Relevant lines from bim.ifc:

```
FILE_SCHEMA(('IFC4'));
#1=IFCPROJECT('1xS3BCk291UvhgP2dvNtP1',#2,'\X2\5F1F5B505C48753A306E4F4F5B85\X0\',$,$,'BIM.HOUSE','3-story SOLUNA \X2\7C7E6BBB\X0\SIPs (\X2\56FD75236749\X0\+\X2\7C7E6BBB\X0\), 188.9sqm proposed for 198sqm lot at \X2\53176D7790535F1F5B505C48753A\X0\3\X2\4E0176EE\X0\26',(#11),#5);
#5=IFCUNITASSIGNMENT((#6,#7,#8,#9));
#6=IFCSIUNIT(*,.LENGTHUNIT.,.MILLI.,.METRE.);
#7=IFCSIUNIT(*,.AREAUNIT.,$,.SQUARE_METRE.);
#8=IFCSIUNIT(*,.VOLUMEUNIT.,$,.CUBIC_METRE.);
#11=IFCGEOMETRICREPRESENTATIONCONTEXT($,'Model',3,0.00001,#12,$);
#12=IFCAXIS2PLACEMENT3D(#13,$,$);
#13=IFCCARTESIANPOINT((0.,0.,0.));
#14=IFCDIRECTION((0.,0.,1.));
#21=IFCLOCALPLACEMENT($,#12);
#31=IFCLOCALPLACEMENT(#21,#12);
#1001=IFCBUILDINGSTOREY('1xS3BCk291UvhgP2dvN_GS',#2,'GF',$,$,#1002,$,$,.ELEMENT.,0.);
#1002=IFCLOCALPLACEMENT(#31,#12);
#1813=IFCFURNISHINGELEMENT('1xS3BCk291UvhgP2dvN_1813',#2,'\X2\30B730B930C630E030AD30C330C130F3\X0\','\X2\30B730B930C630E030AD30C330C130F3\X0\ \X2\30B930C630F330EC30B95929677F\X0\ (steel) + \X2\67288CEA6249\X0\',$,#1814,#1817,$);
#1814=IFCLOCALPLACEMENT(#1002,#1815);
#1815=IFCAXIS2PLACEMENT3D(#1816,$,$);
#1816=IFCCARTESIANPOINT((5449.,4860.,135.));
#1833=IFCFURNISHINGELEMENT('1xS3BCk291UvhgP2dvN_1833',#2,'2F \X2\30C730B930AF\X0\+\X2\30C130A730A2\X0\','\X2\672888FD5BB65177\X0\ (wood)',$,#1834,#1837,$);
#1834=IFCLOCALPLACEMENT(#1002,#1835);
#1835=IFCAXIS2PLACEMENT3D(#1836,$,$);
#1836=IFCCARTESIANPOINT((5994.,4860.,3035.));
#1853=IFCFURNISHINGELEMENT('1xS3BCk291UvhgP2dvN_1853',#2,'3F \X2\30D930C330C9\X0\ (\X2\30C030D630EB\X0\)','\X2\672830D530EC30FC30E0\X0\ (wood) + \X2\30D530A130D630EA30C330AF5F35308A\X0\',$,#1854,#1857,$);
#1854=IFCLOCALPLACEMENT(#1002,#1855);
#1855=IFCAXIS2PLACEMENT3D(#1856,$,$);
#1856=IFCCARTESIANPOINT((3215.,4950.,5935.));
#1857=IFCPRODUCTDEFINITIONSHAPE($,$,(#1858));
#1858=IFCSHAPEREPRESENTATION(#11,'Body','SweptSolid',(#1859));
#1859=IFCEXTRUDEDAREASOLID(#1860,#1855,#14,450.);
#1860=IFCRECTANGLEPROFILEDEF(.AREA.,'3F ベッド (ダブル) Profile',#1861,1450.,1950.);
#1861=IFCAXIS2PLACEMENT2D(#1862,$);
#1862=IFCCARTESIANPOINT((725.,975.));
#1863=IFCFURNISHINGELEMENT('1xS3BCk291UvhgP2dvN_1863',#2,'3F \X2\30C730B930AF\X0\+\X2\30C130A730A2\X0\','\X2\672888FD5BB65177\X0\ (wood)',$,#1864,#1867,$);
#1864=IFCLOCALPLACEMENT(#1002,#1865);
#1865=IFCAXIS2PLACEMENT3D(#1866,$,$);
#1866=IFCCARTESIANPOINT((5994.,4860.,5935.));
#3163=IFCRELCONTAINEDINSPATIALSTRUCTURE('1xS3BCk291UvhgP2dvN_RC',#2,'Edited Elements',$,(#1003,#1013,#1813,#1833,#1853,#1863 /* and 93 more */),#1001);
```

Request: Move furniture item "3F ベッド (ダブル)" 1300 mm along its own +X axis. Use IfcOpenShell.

```python
import ifcopenshell
import ifcopenshell.api.geometry
import ifcopenshell.util.placement
import ifcopenshell.util.unit

model = ifcopenshell.open("bim.ifc")
unit_scale = ifcopenshell.util.unit.calculate_unit_scale(model)

item = model.by_guid("1xS3BCk291UvhgP2dvN_1853")
matrix = ifcopenshell.util.placement.get_local_placement(item.ObjectPlacement)
matrix[:3, 3] += matrix[:3, 0] * 1.3 / unit_scale
ifcopenshell.api.geometry.edit_object_placement(model, product=item, matrix=matrix, is_si=False)

print(ifcopenshell.util.placement.get_local_placement(item.ObjectPlacement).round(3) + 0.0)

model.write("bim_rev.ifc")
```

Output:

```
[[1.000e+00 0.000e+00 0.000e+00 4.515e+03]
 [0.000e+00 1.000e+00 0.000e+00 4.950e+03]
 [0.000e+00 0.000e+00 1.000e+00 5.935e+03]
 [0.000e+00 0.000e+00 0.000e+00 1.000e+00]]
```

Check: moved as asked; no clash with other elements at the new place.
